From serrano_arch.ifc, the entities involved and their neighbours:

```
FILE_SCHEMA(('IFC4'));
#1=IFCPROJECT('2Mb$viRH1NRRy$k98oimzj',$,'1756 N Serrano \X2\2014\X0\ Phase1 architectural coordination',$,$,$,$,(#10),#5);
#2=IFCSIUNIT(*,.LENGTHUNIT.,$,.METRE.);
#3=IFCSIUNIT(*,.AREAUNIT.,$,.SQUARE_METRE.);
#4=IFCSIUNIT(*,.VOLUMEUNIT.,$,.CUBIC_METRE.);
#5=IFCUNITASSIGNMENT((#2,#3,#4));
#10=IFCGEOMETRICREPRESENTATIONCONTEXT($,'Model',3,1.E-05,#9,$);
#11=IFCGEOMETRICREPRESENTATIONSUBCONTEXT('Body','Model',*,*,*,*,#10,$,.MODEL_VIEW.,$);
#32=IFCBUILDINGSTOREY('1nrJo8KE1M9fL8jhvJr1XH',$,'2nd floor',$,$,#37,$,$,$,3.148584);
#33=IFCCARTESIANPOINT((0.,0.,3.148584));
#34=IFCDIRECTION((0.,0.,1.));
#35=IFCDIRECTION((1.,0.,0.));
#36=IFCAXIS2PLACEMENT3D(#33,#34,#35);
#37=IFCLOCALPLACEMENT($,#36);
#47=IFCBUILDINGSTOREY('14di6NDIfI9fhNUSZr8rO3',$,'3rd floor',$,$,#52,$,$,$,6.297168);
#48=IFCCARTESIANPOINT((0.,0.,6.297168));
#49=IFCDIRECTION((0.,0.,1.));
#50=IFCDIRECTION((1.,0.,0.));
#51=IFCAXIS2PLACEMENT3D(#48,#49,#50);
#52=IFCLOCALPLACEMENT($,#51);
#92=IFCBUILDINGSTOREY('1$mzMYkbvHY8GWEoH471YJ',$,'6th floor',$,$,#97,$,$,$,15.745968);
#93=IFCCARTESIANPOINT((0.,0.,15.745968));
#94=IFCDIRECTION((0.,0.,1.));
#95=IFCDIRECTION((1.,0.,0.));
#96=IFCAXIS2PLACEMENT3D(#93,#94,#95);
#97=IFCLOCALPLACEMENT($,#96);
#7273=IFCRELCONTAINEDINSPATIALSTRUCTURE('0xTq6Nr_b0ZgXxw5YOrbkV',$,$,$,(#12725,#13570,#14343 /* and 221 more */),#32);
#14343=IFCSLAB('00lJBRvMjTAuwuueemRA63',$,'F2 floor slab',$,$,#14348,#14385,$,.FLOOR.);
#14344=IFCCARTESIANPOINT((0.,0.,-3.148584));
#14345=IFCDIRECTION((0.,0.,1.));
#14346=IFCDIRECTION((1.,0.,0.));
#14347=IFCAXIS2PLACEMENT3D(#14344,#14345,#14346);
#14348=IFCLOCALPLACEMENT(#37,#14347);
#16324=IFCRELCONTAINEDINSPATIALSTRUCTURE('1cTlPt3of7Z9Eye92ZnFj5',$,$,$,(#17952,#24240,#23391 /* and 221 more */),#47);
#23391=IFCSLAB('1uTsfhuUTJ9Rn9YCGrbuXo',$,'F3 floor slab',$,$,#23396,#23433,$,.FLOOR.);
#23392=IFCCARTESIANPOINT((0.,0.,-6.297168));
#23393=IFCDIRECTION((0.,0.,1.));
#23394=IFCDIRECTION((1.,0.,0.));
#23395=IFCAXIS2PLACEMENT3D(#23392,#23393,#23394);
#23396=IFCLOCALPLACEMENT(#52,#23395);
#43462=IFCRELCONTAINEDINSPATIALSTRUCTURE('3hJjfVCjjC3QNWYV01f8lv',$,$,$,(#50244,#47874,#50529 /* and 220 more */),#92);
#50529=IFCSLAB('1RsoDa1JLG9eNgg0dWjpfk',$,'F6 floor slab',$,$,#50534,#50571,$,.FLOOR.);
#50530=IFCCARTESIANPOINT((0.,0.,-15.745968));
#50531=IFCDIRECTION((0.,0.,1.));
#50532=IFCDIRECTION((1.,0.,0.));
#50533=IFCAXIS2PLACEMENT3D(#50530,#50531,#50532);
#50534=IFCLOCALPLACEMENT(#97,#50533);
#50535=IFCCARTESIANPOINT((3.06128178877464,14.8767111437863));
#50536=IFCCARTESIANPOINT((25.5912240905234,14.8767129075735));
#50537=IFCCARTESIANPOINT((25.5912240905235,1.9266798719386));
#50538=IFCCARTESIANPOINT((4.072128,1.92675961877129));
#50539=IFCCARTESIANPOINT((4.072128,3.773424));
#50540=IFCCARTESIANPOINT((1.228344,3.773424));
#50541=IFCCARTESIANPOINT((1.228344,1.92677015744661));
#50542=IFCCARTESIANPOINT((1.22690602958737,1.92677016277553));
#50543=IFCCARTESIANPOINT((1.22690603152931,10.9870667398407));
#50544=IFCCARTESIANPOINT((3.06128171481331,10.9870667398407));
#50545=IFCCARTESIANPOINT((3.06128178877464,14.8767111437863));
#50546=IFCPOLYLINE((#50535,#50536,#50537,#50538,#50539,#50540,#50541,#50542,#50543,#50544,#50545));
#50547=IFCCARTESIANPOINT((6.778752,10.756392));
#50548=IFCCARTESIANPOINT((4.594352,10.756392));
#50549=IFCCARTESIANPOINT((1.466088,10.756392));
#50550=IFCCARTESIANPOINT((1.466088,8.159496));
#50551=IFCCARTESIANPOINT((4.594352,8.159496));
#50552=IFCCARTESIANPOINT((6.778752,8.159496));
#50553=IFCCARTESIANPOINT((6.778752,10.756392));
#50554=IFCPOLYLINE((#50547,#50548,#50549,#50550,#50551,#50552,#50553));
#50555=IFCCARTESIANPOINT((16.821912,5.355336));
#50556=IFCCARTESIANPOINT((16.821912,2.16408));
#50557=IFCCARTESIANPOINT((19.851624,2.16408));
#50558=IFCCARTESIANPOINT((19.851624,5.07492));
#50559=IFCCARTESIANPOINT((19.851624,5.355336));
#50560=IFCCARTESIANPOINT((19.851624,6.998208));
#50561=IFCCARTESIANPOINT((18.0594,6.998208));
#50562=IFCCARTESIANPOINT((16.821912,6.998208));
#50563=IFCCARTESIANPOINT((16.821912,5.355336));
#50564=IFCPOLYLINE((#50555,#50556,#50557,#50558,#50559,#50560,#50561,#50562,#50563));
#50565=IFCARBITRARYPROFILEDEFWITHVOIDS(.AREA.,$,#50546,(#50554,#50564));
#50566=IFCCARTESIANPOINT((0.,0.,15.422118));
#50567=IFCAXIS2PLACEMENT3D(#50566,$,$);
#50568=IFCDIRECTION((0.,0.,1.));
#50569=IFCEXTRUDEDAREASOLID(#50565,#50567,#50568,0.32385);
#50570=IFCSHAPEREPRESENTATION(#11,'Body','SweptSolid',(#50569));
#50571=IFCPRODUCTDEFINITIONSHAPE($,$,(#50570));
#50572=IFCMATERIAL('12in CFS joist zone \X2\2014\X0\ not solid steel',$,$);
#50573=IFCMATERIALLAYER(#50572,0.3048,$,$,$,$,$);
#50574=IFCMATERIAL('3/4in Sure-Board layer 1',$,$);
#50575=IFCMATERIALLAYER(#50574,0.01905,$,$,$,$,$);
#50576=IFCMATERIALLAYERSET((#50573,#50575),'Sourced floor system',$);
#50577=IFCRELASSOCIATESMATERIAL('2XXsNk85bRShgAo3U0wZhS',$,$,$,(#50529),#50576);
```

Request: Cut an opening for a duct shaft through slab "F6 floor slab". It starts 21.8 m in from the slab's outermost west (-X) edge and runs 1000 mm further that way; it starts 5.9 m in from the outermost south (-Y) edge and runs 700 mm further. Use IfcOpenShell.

```python
import numpy as np
import ifcopenshell
import ifcopenshell.api.feature
import ifcopenshell.api.geometry
import ifcopenshell.api.root
import ifcopenshell.geom
import ifcopenshell.util.placement
import ifcopenshell.util.representation
import ifcopenshell.util.shape
import ifcopenshell.util.unit

model = ifcopenshell.open("serrano_arch.ifc")
unit_scale = ifcopenshell.util.unit.calculate_unit_scale(model)
settings = ifcopenshell.geom.settings()


def volume(element):
    """Net volume in cubic metres, openings subtracted."""
    shape = ifcopenshell.geom.create_shape(settings, element)
    return ifcopenshell.util.shape.get_volume(shape.geometry)


slab = model.by_guid("1RsoDa1JLG9eNgg0dWjpfk")
before = volume(slab)

# Extent in the slab's own axes, in metres. The edges named are its -X and -Y sides.
slab_shape = ifcopenshell.geom.create_shape(settings, slab)
vertices = ifcopenshell.util.shape.get_vertices(slab_shape.geometry)
x_min, y_min, bottom = vertices.min(axis=0)
top = vertices[:, 2].max()

opening = ifcopenshell.api.root.create_entity(model, ifc_class="IfcOpeningElement", name="Duct shaft opening", predefined_type="OPENING")
context = ifcopenshell.util.representation.get_context(model, "Model", "Body", "MODEL_VIEW")
width, depth = 1, 0.7
outline = [(0.0, 0.0), (width, 0.0), (width, depth), (0.0, depth), (0.0, 0.0)]
# Overshoot both faces by 50 mm so the cut is clean.
shape = ifcopenshell.api.geometry.add_slab_representation(
    model, context=context, depth=top - bottom + 0.1, polyline=outline
)
ifcopenshell.api.geometry.assign_representation(model, product=opening, representation=shape)

matrix = ifcopenshell.util.placement.get_local_placement(slab.ObjectPlacement)
matrix[:, 3] = matrix @ np.append(np.array([x_min + 21.8, y_min + 5.9, bottom - 0.05]) / unit_scale, 1.0)
ifcopenshell.api.geometry.edit_object_placement(model, product=opening, matrix=matrix, is_si=False)
ifcopenshell.api.feature.add_feature(model, feature=opening, element=slab)

after = volume(slab)

print(f"slab volume {before:.3f} -> {after:.3f} m3")

model.write("serrano_arch_edited.ifc")
```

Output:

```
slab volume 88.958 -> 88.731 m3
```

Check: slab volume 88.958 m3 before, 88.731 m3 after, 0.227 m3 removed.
